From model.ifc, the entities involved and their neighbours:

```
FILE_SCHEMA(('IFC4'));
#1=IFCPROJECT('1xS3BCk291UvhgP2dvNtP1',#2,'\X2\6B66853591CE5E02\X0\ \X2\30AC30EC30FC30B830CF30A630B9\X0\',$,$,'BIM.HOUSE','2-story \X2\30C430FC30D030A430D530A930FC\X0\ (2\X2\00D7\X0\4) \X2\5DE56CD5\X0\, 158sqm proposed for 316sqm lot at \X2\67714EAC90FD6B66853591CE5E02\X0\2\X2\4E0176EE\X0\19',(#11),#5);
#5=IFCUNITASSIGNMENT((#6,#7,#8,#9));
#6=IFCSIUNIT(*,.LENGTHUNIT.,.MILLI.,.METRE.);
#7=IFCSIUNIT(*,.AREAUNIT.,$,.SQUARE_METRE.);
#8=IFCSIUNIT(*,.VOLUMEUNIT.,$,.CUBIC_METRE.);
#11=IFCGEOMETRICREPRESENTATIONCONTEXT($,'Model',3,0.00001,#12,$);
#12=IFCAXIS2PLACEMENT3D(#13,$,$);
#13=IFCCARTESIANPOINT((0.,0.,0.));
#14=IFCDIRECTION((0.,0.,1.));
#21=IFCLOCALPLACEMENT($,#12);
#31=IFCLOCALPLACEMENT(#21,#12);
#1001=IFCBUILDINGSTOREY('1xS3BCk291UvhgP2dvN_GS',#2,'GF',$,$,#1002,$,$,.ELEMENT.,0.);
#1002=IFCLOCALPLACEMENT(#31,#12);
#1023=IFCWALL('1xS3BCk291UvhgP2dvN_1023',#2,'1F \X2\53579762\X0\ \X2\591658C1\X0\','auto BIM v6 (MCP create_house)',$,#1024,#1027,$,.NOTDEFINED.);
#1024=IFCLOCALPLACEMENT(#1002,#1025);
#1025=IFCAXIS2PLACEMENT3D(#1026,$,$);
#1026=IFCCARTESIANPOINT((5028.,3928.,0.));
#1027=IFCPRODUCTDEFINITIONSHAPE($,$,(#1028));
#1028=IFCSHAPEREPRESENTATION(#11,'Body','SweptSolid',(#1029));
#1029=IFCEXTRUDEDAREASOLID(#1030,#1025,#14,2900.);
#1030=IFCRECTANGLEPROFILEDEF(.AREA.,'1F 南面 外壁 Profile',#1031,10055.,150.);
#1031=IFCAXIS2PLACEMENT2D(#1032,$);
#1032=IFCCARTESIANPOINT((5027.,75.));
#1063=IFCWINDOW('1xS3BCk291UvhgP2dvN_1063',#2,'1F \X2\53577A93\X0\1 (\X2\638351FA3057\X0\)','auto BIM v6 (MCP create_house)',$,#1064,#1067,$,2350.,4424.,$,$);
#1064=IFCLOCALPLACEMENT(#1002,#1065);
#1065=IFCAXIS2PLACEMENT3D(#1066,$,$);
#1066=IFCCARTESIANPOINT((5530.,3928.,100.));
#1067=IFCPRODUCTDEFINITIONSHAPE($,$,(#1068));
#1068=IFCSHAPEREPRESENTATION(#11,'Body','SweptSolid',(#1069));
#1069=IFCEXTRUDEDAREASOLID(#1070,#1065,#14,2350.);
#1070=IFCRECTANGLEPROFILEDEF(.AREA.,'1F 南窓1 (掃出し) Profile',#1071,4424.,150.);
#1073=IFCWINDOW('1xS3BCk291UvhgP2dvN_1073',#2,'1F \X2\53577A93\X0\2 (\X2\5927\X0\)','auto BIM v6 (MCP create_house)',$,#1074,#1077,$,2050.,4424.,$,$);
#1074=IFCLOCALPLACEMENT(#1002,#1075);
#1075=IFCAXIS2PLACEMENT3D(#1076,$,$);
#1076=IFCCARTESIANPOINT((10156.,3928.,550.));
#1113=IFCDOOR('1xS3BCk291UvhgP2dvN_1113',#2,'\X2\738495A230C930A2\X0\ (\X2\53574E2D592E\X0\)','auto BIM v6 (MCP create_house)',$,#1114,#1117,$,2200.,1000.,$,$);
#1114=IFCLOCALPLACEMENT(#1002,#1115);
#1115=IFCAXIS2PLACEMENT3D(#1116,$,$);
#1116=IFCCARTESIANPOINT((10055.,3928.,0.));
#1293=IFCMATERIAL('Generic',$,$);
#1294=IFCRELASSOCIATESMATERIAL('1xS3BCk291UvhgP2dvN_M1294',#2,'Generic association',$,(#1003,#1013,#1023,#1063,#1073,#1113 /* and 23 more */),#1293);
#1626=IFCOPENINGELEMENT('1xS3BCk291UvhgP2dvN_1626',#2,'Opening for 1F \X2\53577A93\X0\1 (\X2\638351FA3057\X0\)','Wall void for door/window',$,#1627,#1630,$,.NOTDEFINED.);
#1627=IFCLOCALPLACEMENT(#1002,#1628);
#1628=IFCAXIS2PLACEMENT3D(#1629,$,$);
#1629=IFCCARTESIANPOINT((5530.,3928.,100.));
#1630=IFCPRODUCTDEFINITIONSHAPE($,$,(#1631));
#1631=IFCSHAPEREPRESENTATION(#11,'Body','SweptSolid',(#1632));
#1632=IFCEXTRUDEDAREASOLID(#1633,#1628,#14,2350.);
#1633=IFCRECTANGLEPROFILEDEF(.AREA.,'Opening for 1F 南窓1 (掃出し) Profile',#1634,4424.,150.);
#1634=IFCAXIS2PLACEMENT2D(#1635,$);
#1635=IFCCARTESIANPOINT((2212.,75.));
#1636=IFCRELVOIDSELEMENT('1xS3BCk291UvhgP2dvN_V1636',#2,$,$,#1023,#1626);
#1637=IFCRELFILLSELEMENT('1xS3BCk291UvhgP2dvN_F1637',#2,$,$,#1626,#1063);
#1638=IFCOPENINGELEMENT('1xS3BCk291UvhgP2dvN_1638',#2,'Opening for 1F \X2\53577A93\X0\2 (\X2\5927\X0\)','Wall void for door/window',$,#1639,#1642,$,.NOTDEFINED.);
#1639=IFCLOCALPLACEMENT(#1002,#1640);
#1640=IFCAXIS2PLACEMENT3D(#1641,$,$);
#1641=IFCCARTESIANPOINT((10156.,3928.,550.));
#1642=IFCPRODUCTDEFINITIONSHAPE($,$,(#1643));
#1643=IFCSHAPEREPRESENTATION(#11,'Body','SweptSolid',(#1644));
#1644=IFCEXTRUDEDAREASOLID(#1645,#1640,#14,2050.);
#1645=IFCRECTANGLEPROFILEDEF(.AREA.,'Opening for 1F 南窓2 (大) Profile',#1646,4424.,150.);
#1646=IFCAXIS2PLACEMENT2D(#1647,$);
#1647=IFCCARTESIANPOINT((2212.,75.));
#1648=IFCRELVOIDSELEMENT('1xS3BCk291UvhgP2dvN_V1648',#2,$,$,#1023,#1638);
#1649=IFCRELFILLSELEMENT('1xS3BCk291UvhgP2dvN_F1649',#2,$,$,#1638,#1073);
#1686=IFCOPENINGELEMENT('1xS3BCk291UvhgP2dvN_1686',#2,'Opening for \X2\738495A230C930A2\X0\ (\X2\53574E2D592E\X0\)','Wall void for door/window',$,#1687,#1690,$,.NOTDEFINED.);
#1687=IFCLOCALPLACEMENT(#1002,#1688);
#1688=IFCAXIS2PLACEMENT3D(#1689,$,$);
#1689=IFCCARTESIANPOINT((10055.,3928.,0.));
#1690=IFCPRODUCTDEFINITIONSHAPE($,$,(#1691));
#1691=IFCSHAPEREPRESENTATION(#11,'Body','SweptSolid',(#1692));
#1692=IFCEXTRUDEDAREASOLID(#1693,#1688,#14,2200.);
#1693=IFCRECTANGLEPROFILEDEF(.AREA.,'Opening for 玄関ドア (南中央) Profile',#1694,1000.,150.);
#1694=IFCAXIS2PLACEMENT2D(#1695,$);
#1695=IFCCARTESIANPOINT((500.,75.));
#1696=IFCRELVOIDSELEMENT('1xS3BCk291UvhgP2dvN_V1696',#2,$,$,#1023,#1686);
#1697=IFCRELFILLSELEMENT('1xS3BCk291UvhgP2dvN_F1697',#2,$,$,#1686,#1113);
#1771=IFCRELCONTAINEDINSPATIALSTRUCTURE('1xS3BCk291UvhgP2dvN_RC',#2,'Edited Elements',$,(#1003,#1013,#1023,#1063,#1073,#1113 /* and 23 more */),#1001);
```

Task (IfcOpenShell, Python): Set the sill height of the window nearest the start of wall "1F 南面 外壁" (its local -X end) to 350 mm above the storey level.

```python
import numpy as np
import ifcopenshell
import ifcopenshell.api.geometry
import ifcopenshell.geom
import ifcopenshell.util.element
import ifcopenshell.util.placement
import ifcopenshell.util.shape
import ifcopenshell.util.unit

model = ifcopenshell.open("model.ifc")
unit_scale = ifcopenshell.util.unit.calculate_unit_scale(model)

window = model.by_id(1063)
opening = window.FillsVoids[0].RelatingOpeningElement
storey = ifcopenshell.util.element.get_container(window, ifc_class="IfcBuildingStorey")
level = ifcopenshell.util.placement.get_local_placement(storey.ObjectPlacement)[2, 3]

# The opening's origin need not be at the sill, so measure its lowest point.
shape = ifcopenshell.geom.create_shape(ifcopenshell.geom.settings(), opening)
bottom = ifcopenshell.util.shape.get_shape_bottom_elevation(shape, shape.geometry) / unit_scale
dz = level + 0.35 / unit_scale - bottom

shift = np.array([0.0, 0.0, dz])
# The window is not placed relative to its opening, so move both.
for product in (opening, window):
    matrix = ifcopenshell.util.placement.get_local_placement(product.ObjectPlacement)
    matrix[:3, 3] += shift
    ifcopenshell.api.geometry.edit_object_placement(model, product=product, matrix=matrix, is_si=False)

print(f"moved by {dz * unit_scale:+.3f} m")

model.write("model_updated.ifc")
```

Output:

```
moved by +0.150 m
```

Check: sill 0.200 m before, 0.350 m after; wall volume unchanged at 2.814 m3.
